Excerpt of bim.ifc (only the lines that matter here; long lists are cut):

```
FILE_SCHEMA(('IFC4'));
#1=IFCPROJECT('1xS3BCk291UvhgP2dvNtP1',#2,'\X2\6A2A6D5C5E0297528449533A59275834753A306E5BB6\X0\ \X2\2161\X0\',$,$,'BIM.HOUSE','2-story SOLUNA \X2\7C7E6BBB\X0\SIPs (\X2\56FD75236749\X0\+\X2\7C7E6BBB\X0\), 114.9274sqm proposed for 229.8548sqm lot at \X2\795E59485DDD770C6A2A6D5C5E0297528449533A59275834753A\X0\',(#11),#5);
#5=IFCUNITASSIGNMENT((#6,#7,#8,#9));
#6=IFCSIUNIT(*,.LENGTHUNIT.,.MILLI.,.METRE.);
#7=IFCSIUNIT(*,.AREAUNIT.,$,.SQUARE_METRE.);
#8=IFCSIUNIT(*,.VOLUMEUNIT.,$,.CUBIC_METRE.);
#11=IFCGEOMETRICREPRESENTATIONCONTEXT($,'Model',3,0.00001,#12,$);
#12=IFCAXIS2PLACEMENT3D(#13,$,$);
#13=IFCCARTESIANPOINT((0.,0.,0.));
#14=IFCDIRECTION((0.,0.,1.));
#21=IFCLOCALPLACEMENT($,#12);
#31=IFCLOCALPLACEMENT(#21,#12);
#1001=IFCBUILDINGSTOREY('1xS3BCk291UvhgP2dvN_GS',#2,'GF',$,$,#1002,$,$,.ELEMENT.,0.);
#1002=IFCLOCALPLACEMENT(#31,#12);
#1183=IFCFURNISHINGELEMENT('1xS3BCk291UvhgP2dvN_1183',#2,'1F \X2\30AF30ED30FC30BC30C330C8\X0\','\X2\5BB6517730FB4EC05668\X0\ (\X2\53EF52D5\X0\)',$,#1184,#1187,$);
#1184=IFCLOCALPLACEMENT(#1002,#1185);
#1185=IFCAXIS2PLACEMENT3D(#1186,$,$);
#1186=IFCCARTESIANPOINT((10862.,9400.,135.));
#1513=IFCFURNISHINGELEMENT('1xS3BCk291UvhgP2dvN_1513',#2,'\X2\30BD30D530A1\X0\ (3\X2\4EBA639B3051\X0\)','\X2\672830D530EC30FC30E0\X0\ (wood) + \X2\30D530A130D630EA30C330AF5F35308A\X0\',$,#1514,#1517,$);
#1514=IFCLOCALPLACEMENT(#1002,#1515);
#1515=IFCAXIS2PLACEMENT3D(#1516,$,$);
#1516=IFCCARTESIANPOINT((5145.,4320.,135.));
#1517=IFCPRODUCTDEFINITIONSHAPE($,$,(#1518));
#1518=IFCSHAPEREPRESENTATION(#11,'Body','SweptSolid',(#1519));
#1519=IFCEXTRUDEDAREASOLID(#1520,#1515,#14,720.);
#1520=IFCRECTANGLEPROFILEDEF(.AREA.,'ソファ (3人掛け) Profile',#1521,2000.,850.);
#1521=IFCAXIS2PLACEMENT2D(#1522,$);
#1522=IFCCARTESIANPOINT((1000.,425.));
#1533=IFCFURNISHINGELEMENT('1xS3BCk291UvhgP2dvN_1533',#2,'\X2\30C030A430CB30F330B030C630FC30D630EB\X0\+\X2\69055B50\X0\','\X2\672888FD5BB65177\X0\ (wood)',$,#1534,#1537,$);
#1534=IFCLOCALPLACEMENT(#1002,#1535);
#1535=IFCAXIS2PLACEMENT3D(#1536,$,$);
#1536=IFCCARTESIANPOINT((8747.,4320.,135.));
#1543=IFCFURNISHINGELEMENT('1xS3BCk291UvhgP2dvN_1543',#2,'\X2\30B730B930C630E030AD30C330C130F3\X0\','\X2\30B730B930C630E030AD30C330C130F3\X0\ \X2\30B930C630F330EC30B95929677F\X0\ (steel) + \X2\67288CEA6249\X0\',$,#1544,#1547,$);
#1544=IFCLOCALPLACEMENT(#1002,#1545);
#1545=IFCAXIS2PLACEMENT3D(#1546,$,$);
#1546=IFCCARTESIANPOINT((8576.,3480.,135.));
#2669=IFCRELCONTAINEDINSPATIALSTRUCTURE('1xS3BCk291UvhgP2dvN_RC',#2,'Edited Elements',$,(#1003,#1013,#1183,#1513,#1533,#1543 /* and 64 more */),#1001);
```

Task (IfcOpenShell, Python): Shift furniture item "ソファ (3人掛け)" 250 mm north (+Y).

```python
import ifcopenshell
import ifcopenshell.api.geometry
import ifcopenshell.util.placement
import ifcopenshell.util.unit

model = ifcopenshell.open("bim.ifc")
unit_scale = ifcopenshell.util.unit.calculate_unit_scale(model)

item = model.by_guid("1xS3BCk291UvhgP2dvN_1513")
matrix = ifcopenshell.util.placement.get_local_placement(item.ObjectPlacement)
matrix[1, 3] += 0.25 / unit_scale
ifcopenshell.api.geometry.edit_object_placement(model, product=item, matrix=matrix, is_si=False)

print(ifcopenshell.util.placement.get_local_placement(item.ObjectPlacement).round(3) + 0.0)

model.write("bim-out.ifc")
```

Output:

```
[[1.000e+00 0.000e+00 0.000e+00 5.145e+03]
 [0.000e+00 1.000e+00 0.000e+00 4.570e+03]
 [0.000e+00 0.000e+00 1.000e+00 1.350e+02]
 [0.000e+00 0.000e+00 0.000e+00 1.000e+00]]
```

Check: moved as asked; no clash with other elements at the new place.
